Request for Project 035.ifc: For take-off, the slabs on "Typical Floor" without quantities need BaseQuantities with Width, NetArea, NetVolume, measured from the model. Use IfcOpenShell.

First a look at what the model holds.

```python
import ifcopenshell
import ifcopenshell.util.element
import ifcopenshell.util.unit

model = ifcopenshell.open("Project 035.ifc")
print(model.schema)
for unit_type in ("LENGTHUNIT", "AREAUNIT", "VOLUMEUNIT"):
    print(unit_type, ifcopenshell.util.unit.calculate_unit_scale(model, unit_type))
storey = next(s for s in model.by_type("IfcBuildingStorey") if s.Name == "Typical Floor")
slabs = [e for e in ifcopenshell.util.element.get_decomposition(storey) if e.is_a("IfcSlab")]
for e in sorted(slabs, key=lambda e: e.id()):
    print(e.id(), e.is_a(), e.Name, list(ifcopenshell.util.element.get_psets(e, qtos_only=True)), sep=" | ")
```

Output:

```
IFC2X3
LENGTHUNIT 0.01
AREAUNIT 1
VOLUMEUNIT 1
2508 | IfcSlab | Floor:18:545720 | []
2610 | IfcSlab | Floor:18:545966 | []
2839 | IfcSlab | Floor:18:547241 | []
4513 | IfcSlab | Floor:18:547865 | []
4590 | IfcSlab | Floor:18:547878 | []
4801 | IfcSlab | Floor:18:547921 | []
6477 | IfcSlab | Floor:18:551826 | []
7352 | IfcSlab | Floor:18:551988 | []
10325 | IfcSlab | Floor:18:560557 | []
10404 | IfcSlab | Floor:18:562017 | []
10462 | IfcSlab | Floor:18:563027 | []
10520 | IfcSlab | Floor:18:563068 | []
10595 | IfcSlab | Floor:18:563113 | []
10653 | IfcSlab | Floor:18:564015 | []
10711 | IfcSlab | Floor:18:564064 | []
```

```python
import ifcopenshell
import ifcopenshell.api.pset
import ifcopenshell.geom
import ifcopenshell.util.element
import ifcopenshell.util.shape
import ifcopenshell.util.unit

model = ifcopenshell.open("Project 035.ifc")
unit_scale = ifcopenshell.util.unit.calculate_unit_scale(model)
area_scale = ifcopenshell.util.unit.calculate_unit_scale(model, "AREAUNIT")
volume_scale = ifcopenshell.util.unit.calculate_unit_scale(model, "VOLUMEUNIT")
settings = ifcopenshell.geom.settings()

storey = next(s for s in model.by_type("IfcBuildingStorey") if s.Name == "Typical Floor")
slabs = [e for e in ifcopenshell.util.element.get_decomposition(storey) if e.is_a("IfcSlab")]

for e in sorted(slabs, key=lambda e: e.id()):
    if ifcopenshell.util.element.get_psets(e, qtos_only=True, should_inherit=False):
        continue
    # Geometry comes back in metres, in the element's own axes.
    shape = ifcopenshell.geom.create_shape(settings, e)
    values = {
        "Width": ifcopenshell.util.shape.get_z(shape.geometry) / unit_scale,
        "NetArea": ifcopenshell.util.shape.get_footprint_area(shape.geometry) / area_scale,
        "NetVolume": ifcopenshell.util.shape.get_volume(shape.geometry) / volume_scale,
    }
    qto = ifcopenshell.api.pset.add_qto(model, product=e, name="BaseQuantities")
    ifcopenshell.api.pset.edit_qto(model, qto=qto, properties=values)
    print(e.id(), {k: round(v, 3) for k, v in values.items()})

model.write("Project 035_rev.ifc")
```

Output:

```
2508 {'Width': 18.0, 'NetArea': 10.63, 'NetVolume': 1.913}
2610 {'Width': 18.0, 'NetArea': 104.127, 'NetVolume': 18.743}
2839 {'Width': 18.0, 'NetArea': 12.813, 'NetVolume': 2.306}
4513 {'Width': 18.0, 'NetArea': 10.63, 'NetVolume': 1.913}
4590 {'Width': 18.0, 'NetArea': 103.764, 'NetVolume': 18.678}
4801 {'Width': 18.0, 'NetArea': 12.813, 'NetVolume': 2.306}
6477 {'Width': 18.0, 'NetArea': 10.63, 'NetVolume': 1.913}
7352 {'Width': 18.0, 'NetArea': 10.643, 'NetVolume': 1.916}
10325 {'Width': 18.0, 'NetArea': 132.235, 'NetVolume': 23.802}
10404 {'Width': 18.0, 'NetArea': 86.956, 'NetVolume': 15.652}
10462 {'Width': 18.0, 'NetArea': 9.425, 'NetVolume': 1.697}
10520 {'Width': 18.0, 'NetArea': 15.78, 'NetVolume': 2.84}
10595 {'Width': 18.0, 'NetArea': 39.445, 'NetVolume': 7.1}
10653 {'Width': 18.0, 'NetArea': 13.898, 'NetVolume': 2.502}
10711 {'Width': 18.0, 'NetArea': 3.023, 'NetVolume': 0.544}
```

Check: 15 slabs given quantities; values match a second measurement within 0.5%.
